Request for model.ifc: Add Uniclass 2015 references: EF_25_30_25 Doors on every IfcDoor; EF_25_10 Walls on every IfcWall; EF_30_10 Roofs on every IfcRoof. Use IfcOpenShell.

First a look at what the model holds.

```python
import ifcopenshell

model = ifcopenshell.open("model.ifc")
print(model.schema)
print("classifications:", [c.Name for c in model.by_type("IfcClassification")])
for ifc_class in ("IfcDoor", "IfcRoof", "IfcStair", "IfcWall", "IfcWindow"):
    print(ifc_class, len(model.by_type(ifc_class)))
```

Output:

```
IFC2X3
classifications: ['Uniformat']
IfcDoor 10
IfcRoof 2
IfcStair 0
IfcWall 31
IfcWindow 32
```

```python
import ifcopenshell
import ifcopenshell.api.classification

model = ifcopenshell.open("model.ifc")

# IFC2X3 requires Source and Edition and has no link from the project to the system.
system = model.create_entity("IfcClassification", Source="NBS", Edition="2015", Name="Uniclass 2015")

codes = {
    "IfcDoor": ("EF_25_30_25", "Doors"),
    "IfcWall": ("EF_25_10", "Walls"),
    "IfcRoof": ("EF_30_10", "Roofs"),
}
for ifc_class, (code, name) in codes.items():
    products = model.by_type(ifc_class)
    ifcopenshell.api.classification.add_reference(
        model, products=products, classification=system, identification=code, name=name
    )
    print(code, len(products))

model.write("model_rev.ifc")
```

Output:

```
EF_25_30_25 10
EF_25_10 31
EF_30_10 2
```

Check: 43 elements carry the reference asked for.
